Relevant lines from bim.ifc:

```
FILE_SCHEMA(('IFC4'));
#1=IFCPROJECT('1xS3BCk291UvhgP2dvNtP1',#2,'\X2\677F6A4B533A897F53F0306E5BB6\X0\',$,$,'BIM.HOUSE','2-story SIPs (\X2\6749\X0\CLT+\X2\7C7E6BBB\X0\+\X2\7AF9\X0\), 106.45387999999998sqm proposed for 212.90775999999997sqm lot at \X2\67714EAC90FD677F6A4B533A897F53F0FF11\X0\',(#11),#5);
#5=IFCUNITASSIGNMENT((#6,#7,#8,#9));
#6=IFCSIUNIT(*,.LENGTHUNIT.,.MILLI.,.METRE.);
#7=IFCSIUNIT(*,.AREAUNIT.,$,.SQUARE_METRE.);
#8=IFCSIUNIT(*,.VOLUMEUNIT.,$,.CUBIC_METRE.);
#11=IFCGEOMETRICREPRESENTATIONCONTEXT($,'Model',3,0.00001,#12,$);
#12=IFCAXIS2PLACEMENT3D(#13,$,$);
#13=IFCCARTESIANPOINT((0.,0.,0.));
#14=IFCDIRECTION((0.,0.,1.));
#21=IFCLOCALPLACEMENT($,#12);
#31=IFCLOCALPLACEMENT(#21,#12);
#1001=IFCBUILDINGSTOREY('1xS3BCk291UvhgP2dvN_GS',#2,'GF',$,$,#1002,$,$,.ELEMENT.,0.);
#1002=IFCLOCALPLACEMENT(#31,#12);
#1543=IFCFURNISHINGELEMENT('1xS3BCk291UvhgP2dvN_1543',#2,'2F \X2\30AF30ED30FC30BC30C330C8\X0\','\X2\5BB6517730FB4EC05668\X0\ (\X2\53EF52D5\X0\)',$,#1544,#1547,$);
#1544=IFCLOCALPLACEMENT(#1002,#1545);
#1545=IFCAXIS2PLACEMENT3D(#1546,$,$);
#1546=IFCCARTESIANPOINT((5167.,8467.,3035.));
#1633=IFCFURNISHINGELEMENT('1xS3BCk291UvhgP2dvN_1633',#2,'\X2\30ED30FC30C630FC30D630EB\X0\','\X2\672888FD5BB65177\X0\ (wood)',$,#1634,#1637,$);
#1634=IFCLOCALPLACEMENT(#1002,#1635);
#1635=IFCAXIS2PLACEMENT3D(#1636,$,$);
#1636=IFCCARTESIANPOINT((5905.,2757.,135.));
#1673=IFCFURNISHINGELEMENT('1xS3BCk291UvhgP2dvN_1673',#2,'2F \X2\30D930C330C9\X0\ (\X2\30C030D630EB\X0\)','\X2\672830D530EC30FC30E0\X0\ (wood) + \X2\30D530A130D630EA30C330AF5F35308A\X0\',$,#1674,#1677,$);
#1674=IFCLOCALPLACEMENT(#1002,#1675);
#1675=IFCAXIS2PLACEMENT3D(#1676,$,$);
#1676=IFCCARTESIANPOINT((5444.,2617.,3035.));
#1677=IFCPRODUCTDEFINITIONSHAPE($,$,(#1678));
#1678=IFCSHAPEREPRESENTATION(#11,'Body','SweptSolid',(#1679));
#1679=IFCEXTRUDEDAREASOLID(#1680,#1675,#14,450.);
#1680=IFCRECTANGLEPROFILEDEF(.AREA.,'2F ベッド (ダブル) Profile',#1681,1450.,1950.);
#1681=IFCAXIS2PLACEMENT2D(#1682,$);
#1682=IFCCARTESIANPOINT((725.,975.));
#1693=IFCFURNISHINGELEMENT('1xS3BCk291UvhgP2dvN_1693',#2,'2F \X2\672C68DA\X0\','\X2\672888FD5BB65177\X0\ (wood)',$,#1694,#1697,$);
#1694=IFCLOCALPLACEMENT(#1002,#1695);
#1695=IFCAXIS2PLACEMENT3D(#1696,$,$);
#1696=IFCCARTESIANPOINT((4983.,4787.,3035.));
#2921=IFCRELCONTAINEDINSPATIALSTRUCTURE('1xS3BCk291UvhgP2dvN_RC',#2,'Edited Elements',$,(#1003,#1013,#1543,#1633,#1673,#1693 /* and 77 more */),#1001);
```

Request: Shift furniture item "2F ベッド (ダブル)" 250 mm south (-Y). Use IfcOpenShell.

```python
import ifcopenshell
import ifcopenshell.api.geometry
import ifcopenshell.util.placement
import ifcopenshell.util.unit

model = ifcopenshell.open("bim.ifc")
unit_scale = ifcopenshell.util.unit.calculate_unit_scale(model)

item = model.by_guid("1xS3BCk291UvhgP2dvN_1673")
matrix = ifcopenshell.util.placement.get_local_placement(item.ObjectPlacement)
matrix[1, 3] -= 0.25 / unit_scale
ifcopenshell.api.geometry.edit_object_placement(model, product=item, matrix=matrix, is_si=False)

print(ifcopenshell.util.placement.get_local_placement(item.ObjectPlacement).round(3) + 0.0)

model.write("bim_rev.ifc")
```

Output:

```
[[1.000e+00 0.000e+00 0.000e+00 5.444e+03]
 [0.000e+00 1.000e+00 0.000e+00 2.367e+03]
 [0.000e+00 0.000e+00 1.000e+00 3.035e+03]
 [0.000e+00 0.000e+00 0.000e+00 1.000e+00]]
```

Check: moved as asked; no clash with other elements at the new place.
